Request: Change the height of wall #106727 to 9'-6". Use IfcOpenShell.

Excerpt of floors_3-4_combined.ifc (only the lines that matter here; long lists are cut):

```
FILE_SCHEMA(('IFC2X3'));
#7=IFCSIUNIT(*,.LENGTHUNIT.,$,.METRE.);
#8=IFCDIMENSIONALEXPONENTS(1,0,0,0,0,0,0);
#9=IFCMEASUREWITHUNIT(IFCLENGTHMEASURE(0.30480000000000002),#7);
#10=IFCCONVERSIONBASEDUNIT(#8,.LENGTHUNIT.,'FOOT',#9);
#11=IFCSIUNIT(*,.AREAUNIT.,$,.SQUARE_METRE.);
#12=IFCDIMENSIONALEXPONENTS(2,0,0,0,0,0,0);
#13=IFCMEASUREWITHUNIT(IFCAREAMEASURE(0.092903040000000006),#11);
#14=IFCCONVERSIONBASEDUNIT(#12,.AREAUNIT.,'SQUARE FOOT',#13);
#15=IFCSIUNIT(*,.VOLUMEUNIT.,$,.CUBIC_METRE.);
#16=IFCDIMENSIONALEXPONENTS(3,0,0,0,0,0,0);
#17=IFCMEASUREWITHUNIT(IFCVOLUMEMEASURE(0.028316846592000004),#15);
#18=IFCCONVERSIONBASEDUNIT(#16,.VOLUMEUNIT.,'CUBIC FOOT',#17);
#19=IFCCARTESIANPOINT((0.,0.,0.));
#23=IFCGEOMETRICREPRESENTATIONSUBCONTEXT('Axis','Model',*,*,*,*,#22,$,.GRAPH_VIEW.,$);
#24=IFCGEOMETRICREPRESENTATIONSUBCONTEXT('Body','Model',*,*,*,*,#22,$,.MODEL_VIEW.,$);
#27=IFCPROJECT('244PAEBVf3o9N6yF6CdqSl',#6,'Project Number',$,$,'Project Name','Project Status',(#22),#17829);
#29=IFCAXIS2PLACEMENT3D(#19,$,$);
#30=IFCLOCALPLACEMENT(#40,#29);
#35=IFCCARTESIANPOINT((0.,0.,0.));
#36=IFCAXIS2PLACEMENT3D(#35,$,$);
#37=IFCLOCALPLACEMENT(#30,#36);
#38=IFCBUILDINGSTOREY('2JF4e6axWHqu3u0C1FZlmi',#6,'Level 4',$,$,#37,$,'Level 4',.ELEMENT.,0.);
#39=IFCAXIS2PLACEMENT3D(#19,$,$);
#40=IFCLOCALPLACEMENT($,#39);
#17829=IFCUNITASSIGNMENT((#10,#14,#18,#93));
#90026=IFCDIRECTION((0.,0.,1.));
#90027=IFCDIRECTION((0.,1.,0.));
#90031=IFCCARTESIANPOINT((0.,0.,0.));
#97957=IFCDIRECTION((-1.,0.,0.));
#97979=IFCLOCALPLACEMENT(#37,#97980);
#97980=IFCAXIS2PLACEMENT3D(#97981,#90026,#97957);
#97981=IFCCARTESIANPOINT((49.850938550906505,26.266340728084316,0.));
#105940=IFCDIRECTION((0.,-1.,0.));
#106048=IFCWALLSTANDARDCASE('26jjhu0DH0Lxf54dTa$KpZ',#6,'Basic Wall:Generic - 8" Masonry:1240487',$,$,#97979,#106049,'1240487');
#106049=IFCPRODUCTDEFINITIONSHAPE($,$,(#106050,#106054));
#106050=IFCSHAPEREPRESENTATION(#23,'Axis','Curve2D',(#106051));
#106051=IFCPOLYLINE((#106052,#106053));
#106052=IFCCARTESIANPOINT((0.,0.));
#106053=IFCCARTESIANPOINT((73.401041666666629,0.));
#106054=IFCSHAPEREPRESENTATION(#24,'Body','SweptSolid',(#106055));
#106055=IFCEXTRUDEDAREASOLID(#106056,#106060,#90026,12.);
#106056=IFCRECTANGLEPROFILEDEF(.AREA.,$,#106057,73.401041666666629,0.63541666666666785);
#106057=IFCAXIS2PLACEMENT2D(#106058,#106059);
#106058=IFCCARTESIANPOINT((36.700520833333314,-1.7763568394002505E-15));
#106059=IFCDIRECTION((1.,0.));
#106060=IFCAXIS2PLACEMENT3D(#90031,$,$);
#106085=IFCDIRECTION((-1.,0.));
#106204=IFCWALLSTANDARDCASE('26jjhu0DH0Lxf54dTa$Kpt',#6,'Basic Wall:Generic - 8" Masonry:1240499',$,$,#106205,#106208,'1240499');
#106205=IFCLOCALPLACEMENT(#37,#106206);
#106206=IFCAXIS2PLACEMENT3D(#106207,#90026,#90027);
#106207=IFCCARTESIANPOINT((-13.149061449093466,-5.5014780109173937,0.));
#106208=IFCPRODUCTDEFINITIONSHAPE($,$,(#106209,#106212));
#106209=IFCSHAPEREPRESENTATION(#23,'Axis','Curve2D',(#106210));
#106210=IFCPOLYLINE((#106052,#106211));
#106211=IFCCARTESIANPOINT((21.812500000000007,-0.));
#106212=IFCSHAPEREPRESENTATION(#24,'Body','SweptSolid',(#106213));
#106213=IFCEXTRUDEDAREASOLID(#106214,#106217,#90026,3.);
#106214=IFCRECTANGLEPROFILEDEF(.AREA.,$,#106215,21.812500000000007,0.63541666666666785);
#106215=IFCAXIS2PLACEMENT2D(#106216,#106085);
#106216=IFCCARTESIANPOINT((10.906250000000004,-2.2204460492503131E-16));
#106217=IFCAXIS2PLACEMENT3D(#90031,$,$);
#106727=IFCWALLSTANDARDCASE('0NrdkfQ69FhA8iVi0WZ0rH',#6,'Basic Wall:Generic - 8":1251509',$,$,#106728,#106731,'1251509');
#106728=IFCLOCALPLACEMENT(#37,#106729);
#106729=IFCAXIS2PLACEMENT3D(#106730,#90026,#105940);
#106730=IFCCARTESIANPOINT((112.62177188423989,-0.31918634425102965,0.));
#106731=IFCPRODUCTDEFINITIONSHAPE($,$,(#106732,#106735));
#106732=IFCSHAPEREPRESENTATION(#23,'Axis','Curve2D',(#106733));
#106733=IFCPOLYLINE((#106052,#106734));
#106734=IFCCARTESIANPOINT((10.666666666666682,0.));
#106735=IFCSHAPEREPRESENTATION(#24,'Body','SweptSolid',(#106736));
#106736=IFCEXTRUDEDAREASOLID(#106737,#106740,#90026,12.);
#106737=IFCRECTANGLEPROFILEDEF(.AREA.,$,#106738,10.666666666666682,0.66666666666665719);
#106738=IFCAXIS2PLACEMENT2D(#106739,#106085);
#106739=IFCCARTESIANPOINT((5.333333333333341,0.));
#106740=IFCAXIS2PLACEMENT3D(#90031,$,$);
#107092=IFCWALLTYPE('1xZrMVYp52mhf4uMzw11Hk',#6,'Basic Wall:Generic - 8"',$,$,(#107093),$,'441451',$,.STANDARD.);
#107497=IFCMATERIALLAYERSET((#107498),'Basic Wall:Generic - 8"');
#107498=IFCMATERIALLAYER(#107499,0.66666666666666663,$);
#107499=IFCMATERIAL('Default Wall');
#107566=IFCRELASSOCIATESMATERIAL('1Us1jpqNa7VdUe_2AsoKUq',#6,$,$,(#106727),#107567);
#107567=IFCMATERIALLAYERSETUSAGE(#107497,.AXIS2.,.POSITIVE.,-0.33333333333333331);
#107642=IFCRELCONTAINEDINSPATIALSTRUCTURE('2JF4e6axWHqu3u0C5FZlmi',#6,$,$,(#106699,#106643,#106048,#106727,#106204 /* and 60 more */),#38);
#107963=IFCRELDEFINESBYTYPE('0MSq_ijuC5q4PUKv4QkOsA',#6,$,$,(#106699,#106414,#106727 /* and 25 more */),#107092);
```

```python
import ifcopenshell
import ifcopenshell.geom
import ifcopenshell.util.representation
import ifcopenshell.util.shape
import ifcopenshell.util.unit

model = ifcopenshell.open("floors_3-4_combined.ifc")
unit_scale = ifcopenshell.util.unit.calculate_unit_scale(model)
settings = ifcopenshell.geom.settings()


def volume(element):
    """Net volume in cubic metres, openings subtracted."""
    shape = ifcopenshell.geom.create_shape(settings, element)
    return ifcopenshell.util.shape.get_volume(shape.geometry)


wall = model.by_guid("0NrdkfQ69FhA8iVi0WZ0rH")
before = volume(wall)

body = ifcopenshell.util.representation.get_representation(wall, "Model", "Body")
solid = body.Items[0]
old_height = solid.Depth
solid.Depth = 114 * 0.0254 / unit_scale
after = volume(wall)

print(f"height {old_height:g} -> {solid.Depth:g}, volume {before:.3f} -> {after:.3f} m3")

model.write("floors_3-4_combined_edited.ifc")
```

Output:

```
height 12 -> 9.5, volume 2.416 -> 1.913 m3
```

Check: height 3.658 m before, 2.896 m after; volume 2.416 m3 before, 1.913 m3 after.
